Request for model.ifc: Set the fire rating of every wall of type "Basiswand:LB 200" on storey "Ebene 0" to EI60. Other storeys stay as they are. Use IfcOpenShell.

First a look at what the model holds.

```python
import ifcopenshell
import ifcopenshell.util.element

model = ifcopenshell.open("model.ifc")
print(model.schema)
storey = next(s for s in model.by_type("IfcBuildingStorey") if s.Name == "Ebene 0")
walls = [e for e in ifcopenshell.util.element.get_decomposition(storey) if e.is_a("IfcWall")]
seen = {}
for e in walls:
    element_type = ifcopenshell.util.element.get_type(e)
    key = (element_type.Name if element_type != e and element_type else None, ifcopenshell.util.element.get_pset(e, "Pset_WallCommon", "FireRating"))
    seen[key] = seen.get(key, 0) + 1
for (name, value), count in sorted(seen.items(), key=str):
    print(count, "x", name, "|", value)
```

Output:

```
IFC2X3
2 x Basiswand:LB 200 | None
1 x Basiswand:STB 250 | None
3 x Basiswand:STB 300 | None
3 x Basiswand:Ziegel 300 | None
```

```python
import ifcopenshell
import ifcopenshell.api.pset
import ifcopenshell.util.element

model = ifcopenshell.open("model.ifc")

storey = next(s for s in model.by_type("IfcBuildingStorey") if s.Name == "Ebene 0")
walls = [e for e in ifcopenshell.util.element.get_decomposition(storey) if e.is_a("IfcWall")]

count = 0
for e in walls:
    element_type = ifcopenshell.util.element.get_type(e)
    if element_type in (None, e) or element_type.Name != "Basiswand:LB 200":
        continue
    # add_pset returns the element's existing set when there is one.
    pset = ifcopenshell.api.pset.add_pset(model, product=e, name="Pset_WallCommon")
    ifcopenshell.api.pset.edit_pset(model, pset=pset, properties={"FireRating": "EI60"})
    count += 1

print(count, "walls updated")

model.write("model_updated.ifc")
```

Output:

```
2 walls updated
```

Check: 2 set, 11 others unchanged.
